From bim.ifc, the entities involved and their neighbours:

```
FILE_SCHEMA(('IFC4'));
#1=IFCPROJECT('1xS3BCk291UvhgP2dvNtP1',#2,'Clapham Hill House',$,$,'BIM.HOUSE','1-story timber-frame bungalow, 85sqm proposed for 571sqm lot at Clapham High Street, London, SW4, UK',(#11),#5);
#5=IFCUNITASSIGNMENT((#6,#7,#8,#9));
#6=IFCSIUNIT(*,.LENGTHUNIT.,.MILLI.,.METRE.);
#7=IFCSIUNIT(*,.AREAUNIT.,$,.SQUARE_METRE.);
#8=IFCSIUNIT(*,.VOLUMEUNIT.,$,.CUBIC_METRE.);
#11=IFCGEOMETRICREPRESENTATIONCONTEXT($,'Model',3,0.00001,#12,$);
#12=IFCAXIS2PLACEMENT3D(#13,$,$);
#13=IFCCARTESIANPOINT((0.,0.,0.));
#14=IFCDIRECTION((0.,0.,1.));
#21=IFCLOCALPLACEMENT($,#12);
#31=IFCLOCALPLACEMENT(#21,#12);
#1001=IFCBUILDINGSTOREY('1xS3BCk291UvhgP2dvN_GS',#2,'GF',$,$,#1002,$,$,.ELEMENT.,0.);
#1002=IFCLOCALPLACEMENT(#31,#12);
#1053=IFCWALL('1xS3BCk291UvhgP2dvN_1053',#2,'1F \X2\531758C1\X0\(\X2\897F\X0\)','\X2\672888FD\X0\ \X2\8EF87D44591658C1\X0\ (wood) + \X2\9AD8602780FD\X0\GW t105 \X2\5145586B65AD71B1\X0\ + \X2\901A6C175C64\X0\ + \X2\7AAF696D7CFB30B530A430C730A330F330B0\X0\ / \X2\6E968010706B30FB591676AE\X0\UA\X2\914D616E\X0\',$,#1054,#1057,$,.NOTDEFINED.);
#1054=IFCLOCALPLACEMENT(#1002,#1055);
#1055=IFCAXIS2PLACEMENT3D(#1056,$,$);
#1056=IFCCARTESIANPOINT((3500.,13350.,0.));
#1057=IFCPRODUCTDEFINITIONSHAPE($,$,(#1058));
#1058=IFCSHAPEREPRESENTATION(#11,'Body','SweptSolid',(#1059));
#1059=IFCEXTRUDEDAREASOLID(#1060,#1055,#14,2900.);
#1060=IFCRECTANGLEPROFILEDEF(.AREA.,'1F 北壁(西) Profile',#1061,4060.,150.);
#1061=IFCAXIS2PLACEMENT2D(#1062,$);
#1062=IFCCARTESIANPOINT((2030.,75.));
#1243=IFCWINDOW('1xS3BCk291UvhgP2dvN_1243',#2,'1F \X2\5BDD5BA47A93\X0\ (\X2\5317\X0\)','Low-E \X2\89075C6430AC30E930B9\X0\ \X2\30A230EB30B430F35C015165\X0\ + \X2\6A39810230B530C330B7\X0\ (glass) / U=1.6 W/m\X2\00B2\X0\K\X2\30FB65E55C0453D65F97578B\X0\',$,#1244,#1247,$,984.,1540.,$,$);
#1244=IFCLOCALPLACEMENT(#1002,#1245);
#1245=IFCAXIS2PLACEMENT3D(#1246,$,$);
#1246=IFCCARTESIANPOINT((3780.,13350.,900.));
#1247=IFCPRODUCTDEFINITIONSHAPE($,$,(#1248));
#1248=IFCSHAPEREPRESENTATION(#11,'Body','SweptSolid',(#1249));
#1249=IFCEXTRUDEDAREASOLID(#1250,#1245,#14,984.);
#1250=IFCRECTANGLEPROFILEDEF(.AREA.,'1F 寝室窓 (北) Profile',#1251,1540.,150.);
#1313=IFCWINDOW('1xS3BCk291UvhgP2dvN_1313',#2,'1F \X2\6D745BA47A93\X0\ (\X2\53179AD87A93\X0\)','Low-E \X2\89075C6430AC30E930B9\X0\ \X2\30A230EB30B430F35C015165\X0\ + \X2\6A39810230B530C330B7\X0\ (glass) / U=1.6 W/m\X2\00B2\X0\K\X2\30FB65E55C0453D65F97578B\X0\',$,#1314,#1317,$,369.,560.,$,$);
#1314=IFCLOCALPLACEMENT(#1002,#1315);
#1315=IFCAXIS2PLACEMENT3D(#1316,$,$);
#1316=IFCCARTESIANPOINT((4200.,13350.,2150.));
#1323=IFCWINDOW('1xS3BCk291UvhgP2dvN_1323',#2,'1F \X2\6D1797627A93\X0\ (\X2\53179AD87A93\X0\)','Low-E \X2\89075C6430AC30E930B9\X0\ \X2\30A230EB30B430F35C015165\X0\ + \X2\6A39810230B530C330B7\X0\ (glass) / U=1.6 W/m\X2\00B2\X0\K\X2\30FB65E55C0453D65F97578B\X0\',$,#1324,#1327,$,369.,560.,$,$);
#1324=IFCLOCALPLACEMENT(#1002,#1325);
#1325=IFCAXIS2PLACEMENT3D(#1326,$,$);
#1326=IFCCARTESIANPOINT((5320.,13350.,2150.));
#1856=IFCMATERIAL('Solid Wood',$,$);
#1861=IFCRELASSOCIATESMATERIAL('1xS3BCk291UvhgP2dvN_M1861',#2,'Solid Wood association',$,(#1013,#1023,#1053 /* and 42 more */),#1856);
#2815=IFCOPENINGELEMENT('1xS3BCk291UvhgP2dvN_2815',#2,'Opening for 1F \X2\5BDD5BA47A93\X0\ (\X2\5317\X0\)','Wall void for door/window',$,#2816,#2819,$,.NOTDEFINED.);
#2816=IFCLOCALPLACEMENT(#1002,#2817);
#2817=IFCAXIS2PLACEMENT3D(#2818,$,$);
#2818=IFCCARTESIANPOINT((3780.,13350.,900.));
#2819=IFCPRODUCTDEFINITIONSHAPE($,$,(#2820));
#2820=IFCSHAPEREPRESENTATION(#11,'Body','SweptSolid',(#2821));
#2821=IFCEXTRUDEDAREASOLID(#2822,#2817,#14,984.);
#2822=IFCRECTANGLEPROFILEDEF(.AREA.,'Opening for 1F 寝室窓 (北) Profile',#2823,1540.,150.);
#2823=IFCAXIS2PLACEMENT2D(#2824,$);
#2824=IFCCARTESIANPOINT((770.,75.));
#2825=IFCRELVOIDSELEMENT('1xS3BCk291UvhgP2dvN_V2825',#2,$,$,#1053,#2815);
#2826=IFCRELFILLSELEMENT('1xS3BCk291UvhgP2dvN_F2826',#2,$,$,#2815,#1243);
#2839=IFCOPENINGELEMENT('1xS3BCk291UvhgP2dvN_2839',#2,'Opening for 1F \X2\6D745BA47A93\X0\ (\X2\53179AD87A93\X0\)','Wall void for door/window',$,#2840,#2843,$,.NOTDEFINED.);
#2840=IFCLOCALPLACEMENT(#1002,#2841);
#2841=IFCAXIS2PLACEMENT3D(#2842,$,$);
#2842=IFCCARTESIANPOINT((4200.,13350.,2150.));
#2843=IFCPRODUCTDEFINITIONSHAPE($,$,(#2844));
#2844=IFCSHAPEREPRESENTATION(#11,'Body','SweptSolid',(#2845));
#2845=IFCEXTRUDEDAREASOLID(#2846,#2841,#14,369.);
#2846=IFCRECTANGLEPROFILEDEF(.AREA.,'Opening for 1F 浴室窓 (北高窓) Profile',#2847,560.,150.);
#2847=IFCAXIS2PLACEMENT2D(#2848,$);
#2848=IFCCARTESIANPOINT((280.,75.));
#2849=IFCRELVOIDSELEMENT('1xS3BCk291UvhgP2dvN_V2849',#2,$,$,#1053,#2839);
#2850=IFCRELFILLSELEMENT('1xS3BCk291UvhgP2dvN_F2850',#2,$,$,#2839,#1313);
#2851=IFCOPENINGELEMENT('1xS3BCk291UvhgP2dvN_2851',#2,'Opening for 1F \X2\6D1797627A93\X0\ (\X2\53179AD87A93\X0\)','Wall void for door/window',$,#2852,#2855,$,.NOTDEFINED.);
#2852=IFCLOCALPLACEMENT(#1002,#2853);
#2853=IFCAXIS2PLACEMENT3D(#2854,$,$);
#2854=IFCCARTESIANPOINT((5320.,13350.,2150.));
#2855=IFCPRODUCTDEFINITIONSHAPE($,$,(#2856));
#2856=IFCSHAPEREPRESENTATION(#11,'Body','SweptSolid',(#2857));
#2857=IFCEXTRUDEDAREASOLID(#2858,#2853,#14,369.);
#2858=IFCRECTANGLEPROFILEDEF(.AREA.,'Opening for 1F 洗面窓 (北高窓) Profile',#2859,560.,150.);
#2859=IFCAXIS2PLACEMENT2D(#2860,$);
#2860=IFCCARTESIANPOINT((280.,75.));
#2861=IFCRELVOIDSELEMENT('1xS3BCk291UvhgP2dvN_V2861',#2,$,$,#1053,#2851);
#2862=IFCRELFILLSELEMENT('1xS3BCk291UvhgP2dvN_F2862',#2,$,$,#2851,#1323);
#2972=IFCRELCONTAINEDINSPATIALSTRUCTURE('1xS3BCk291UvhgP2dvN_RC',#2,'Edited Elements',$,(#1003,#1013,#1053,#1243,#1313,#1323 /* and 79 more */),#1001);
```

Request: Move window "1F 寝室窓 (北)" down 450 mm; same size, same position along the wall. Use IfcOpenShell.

```python
import numpy as np
import ifcopenshell
import ifcopenshell.api.geometry
import ifcopenshell.util.placement
import ifcopenshell.util.unit

model = ifcopenshell.open("bim.ifc")
unit_scale = ifcopenshell.util.unit.calculate_unit_scale(model)

window = model.by_id(1243)
opening = window.FillsVoids[0].RelatingOpeningElement
dz = -0.45 / unit_scale

shift = np.array([0.0, 0.0, dz])
# The window is not placed relative to its opening, so move both.
for product in (opening, window):
    matrix = ifcopenshell.util.placement.get_local_placement(product.ObjectPlacement)
    matrix[:3, 3] += shift
    ifcopenshell.api.geometry.edit_object_placement(model, product=product, matrix=matrix, is_si=False)

print(f"moved by {dz * unit_scale:+.3f} m")

model.write("bim_updated.ifc")
```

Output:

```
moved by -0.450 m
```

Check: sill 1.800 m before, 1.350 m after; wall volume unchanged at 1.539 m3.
